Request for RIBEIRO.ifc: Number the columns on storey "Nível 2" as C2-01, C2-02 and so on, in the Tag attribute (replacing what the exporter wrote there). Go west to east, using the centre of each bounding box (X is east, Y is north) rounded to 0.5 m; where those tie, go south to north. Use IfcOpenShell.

First a look at what the model holds.

```python
import ifcopenshell
import ifcopenshell.util.element
import ifcopenshell.util.placement

model = ifcopenshell.open("RIBEIRO.ifc")
print(model.schema)
storey = next(s for s in model.by_type("IfcBuildingStorey") if s.Name == "Nível 2")
columns = [e for e in ifcopenshell.util.element.get_decomposition(storey) if e.is_a("IfcColumn")]
for e in sorted(columns, key=lambda e: e.id()):
    origin = ifcopenshell.util.placement.get_local_placement(e.ObjectPlacement)[:3, 3]
    print(e.id(), e.Tag, e.Name, origin.round(2) + 0.0, sep=" | ")
```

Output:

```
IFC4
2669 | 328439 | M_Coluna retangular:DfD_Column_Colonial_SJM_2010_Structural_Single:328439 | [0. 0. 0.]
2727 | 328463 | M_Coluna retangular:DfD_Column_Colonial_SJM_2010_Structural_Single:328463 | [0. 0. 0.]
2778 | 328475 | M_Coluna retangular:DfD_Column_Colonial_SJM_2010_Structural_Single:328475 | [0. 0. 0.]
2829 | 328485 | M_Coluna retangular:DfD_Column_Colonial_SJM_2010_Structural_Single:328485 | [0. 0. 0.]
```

```python
import ifcopenshell
import ifcopenshell.geom
import ifcopenshell.util.element
import ifcopenshell.util.shape

model = ifcopenshell.open("RIBEIRO.ifc")
settings = ifcopenshell.geom.settings()
settings.set("use-world-coords", True)


def centre(element):
    shape = ifcopenshell.geom.create_shape(settings, element)
    return ifcopenshell.util.shape.get_bbox_centroid(shape.geometry)


storey = next(s for s in model.by_type("IfcBuildingStorey") if s.Name == "Nível 2")
columns = [e for e in ifcopenshell.util.element.get_decomposition(storey) if e.is_a("IfcColumn")]

# Insertion points can sit at a corner or the storey origin, so sort by the geometry (in metres).
centres = {e: centre(e) for e in columns}
columns.sort(key=lambda e: (round(centres[e][0] / 0.5), centres[e][1]))

for i, e in enumerate(columns, start=1):
    number = f"C2-{i:02d}"
    e.Tag = number
    print(e.id(), number)

model.write("RIBEIRO_rev.ifc")
```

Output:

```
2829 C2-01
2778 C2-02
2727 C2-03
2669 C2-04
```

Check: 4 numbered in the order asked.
